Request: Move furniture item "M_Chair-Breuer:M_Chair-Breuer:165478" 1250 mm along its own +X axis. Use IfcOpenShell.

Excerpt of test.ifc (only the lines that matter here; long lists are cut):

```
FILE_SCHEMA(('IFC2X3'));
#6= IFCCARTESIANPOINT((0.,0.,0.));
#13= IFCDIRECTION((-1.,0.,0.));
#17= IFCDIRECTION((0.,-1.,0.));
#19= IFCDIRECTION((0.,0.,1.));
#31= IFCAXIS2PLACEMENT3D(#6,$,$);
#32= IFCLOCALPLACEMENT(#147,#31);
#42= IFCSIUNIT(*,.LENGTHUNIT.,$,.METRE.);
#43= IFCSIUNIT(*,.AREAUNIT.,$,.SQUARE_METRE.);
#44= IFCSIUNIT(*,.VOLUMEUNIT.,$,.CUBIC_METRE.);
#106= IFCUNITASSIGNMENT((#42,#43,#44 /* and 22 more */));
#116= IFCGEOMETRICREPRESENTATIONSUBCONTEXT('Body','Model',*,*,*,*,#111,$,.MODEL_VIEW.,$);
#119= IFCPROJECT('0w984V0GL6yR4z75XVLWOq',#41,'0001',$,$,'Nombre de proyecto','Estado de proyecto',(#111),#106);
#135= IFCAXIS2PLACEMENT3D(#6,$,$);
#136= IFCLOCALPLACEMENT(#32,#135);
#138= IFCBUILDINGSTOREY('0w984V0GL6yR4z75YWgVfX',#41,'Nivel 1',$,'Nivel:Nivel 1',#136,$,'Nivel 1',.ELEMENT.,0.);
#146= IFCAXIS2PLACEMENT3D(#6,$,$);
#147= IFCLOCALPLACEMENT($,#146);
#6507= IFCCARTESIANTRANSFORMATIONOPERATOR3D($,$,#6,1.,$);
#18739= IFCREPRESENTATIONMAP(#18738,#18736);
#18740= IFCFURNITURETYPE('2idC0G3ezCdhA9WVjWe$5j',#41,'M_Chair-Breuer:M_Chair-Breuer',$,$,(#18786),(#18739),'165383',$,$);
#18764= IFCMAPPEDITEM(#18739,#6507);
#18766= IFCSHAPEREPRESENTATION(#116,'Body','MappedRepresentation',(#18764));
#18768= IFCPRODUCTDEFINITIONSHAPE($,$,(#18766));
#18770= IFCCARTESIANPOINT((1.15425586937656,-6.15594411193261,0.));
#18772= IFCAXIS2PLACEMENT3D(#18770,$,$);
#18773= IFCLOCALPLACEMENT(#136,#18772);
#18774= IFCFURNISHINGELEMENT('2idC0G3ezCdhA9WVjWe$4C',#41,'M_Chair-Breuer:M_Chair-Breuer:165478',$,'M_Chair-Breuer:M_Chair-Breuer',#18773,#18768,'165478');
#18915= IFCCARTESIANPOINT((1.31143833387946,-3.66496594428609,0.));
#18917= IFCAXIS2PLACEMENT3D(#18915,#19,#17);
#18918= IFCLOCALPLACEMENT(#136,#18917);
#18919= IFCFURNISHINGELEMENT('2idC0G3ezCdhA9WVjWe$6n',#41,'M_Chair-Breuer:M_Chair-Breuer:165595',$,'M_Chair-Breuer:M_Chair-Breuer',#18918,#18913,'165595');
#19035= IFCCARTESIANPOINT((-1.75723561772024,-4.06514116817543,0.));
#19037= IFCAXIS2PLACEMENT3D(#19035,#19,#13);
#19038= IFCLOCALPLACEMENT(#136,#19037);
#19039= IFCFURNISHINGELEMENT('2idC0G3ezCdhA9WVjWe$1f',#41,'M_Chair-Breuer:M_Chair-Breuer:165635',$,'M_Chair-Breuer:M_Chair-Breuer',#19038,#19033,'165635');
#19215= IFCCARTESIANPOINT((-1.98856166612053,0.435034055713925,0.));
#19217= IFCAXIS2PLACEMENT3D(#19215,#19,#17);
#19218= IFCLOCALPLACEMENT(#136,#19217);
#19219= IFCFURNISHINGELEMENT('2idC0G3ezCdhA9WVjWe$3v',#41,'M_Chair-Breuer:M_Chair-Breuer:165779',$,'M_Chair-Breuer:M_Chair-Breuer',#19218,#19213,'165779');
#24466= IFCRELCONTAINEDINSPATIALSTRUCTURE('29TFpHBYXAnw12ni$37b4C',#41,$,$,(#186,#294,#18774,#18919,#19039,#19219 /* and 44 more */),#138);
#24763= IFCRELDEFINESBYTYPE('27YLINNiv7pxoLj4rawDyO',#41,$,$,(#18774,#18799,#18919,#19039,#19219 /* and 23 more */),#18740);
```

```python
import ifcopenshell
import ifcopenshell.api.geometry
import ifcopenshell.util.placement

model = ifcopenshell.open("test.ifc")

item = model.by_guid("2idC0G3ezCdhA9WVjWe$4C")
matrix = ifcopenshell.util.placement.get_local_placement(item.ObjectPlacement)
matrix[:3, 3] += matrix[:3, 0] * 1.25
ifcopenshell.api.geometry.edit_object_placement(model, product=item, matrix=matrix, is_si=False)

print(ifcopenshell.util.placement.get_local_placement(item.ObjectPlacement).round(3) + 0.0)

model.write("test_rev.ifc")
```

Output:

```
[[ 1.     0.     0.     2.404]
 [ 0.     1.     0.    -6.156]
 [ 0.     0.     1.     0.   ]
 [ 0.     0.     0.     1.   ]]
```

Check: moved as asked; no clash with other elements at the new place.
